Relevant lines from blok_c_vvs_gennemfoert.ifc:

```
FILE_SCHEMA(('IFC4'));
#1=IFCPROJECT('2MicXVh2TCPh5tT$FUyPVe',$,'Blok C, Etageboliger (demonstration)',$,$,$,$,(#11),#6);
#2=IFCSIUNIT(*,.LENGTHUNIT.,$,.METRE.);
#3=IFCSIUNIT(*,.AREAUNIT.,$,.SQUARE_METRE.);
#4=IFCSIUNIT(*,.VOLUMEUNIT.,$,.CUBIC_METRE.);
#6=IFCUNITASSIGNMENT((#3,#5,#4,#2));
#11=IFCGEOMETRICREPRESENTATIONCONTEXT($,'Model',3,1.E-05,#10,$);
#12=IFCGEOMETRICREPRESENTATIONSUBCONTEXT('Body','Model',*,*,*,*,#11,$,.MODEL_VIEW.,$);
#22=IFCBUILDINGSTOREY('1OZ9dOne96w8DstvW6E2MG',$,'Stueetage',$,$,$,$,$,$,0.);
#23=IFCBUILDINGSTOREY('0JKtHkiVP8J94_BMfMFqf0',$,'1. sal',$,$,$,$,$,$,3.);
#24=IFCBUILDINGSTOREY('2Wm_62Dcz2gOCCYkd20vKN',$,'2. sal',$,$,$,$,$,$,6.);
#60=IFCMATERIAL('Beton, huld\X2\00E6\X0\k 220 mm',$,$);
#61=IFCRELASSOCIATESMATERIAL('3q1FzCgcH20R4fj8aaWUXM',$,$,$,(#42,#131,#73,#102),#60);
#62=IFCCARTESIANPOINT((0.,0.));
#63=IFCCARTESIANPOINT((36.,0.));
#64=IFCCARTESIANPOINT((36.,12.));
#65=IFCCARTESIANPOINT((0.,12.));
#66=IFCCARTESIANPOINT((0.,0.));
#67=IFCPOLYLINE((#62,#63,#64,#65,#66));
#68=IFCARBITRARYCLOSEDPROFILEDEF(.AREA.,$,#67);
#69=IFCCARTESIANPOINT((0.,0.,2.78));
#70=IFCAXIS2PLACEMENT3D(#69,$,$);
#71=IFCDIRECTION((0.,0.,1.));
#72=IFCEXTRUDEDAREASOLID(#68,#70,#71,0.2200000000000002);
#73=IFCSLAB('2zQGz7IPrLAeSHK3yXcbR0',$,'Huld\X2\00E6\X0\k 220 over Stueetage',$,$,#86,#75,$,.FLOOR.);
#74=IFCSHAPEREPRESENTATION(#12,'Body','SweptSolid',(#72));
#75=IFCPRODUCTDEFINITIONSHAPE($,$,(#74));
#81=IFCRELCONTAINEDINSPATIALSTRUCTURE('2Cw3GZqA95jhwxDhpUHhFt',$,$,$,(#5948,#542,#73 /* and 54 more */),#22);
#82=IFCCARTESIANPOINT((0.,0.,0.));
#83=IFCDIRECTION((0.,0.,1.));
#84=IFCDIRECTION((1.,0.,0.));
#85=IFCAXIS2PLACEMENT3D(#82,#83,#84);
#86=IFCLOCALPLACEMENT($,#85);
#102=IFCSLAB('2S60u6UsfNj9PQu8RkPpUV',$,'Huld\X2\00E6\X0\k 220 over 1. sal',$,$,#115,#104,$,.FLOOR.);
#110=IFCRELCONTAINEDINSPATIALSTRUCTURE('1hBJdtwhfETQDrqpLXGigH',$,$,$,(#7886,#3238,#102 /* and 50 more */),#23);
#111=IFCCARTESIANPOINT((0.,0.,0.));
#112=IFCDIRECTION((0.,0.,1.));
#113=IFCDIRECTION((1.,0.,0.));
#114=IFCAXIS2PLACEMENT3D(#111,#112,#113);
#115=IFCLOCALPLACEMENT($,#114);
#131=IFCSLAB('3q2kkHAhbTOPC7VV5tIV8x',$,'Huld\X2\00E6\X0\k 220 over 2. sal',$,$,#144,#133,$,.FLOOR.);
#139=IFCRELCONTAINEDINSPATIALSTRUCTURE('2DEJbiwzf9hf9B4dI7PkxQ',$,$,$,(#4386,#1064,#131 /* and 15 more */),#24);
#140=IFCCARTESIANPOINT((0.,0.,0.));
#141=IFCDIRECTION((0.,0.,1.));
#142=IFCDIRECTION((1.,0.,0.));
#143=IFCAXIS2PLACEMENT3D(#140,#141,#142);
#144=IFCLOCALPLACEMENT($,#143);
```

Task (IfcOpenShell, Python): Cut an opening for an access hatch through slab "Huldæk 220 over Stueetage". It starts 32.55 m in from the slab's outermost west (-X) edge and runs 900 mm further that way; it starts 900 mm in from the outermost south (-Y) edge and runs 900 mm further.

```python
import numpy as np
import ifcopenshell
import ifcopenshell.api.feature
import ifcopenshell.api.geometry
import ifcopenshell.api.root
import ifcopenshell.geom
import ifcopenshell.util.placement
import ifcopenshell.util.representation
import ifcopenshell.util.shape
import ifcopenshell.util.unit

model = ifcopenshell.open("blok_c_vvs_gennemfoert.ifc")
unit_scale = ifcopenshell.util.unit.calculate_unit_scale(model)
settings = ifcopenshell.geom.settings()


def volume(element):
    """Net volume in cubic metres, openings subtracted."""
    shape = ifcopenshell.geom.create_shape(settings, element)
    return ifcopenshell.util.shape.get_volume(shape.geometry)


slab = model.by_guid("2zQGz7IPrLAeSHK3yXcbR0")
before = volume(slab)

# Extent in the slab's own axes, in metres. The edges named are its -X and -Y sides.
slab_shape = ifcopenshell.geom.create_shape(settings, slab)
vertices = ifcopenshell.util.shape.get_vertices(slab_shape.geometry)
x_min, y_min, bottom = vertices.min(axis=0)
top = vertices[:, 2].max()

opening = ifcopenshell.api.root.create_entity(model, ifc_class="IfcOpeningElement", name="Access hatch opening", predefined_type="OPENING")
context = ifcopenshell.util.representation.get_context(model, "Model", "Body", "MODEL_VIEW")
width, depth = 0.9, 0.9
outline = [(0.0, 0.0), (width, 0.0), (width, depth), (0.0, depth), (0.0, 0.0)]
# Overshoot both faces by 50 mm so the cut is clean.
shape = ifcopenshell.api.geometry.add_slab_representation(
    model, context=context, depth=top - bottom + 0.1, polyline=outline
)
ifcopenshell.api.geometry.assign_representation(model, product=opening, representation=shape)

matrix = ifcopenshell.util.placement.get_local_placement(slab.ObjectPlacement)
matrix[:, 3] = matrix @ np.append(np.array([x_min + 32.55, y_min + 0.9, bottom - 0.05]) / unit_scale, 1.0)
ifcopenshell.api.geometry.edit_object_placement(model, product=opening, matrix=matrix, is_si=False)
ifcopenshell.api.feature.add_feature(model, feature=opening, element=slab)

after = volume(slab)

print(f"slab volume {before:.3f} -> {after:.3f} m3")

model.write("blok_c_vvs_gennemfoert_edited.ifc")
```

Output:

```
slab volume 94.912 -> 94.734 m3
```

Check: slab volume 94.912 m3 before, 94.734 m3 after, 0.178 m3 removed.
